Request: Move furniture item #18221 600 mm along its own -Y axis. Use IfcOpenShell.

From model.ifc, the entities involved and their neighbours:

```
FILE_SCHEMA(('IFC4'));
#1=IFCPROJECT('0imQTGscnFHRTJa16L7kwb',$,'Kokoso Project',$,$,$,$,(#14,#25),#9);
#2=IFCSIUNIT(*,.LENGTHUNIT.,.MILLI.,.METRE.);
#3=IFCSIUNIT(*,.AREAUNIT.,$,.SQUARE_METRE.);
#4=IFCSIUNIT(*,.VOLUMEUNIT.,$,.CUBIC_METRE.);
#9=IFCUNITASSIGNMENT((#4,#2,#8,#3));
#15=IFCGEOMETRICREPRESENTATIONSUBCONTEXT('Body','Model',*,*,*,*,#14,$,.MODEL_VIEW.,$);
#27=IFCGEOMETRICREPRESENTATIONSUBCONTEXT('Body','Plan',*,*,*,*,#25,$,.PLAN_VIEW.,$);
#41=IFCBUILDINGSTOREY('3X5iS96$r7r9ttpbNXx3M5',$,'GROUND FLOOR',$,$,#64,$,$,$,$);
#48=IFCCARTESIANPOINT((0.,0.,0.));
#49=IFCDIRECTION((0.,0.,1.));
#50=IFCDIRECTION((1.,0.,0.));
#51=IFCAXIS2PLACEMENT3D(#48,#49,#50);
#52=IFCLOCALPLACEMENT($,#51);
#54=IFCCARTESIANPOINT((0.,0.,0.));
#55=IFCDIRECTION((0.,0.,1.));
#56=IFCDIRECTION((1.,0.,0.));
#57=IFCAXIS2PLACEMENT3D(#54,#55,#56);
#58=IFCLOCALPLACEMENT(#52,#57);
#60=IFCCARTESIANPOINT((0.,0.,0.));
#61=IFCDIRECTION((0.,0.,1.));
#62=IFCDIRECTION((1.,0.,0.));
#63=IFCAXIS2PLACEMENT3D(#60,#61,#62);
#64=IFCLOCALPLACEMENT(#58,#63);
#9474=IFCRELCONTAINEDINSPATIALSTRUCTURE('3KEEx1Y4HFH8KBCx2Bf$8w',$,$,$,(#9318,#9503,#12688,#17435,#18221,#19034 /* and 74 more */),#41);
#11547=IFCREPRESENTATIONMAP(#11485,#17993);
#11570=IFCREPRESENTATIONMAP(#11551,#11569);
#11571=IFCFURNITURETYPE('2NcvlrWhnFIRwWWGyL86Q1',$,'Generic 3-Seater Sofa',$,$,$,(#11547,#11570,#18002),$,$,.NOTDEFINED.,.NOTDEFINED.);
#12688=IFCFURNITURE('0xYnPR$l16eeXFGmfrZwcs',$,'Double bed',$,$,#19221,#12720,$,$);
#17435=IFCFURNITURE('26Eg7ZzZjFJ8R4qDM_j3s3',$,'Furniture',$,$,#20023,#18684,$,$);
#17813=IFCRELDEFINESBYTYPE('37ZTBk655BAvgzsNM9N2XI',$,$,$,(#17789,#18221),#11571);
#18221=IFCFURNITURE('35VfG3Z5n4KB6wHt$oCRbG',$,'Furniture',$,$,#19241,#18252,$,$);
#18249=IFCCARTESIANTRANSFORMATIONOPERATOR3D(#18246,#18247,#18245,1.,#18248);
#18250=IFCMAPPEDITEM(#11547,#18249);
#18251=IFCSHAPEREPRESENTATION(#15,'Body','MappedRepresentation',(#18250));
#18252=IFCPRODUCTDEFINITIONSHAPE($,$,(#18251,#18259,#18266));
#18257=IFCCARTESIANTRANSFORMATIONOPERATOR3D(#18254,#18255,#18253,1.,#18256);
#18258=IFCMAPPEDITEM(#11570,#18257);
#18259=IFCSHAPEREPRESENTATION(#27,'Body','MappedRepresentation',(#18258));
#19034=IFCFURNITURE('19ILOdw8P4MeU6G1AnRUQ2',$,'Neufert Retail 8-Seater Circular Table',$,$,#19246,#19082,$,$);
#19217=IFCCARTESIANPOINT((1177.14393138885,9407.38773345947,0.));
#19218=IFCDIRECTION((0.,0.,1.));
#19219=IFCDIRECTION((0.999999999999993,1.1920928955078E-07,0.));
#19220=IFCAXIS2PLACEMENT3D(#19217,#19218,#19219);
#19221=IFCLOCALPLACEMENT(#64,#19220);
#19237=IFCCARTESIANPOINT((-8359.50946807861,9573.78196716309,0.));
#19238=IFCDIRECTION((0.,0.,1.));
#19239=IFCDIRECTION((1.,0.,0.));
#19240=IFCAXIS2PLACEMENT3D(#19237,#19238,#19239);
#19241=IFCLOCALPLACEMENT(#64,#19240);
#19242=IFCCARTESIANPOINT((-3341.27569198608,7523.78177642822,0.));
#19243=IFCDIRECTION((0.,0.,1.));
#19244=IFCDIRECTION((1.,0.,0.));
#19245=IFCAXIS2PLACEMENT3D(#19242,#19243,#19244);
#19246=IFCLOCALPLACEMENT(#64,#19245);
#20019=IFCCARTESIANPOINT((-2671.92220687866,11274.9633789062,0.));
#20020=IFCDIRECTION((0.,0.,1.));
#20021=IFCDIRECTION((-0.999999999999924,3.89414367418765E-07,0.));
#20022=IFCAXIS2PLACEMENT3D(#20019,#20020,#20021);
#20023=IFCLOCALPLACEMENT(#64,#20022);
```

```python
import ifcopenshell
import ifcopenshell.api.geometry
import ifcopenshell.util.placement

model = ifcopenshell.open("model.ifc")

item = model.by_id(18221)
matrix = ifcopenshell.util.placement.get_local_placement(item.ObjectPlacement)
matrix[:3, 3] -= matrix[:3, 1] * 600.0
ifcopenshell.api.geometry.edit_object_placement(model, product=item, matrix=matrix, is_si=False)

print(ifcopenshell.util.placement.get_local_placement(item.ObjectPlacement).round(3) + 0.0)

model.write("model_updated.ifc")
```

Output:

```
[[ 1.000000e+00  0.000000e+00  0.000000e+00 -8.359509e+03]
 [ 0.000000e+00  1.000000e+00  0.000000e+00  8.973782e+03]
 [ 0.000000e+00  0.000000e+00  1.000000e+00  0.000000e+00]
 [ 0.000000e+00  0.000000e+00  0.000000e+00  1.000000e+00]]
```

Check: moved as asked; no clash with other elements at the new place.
